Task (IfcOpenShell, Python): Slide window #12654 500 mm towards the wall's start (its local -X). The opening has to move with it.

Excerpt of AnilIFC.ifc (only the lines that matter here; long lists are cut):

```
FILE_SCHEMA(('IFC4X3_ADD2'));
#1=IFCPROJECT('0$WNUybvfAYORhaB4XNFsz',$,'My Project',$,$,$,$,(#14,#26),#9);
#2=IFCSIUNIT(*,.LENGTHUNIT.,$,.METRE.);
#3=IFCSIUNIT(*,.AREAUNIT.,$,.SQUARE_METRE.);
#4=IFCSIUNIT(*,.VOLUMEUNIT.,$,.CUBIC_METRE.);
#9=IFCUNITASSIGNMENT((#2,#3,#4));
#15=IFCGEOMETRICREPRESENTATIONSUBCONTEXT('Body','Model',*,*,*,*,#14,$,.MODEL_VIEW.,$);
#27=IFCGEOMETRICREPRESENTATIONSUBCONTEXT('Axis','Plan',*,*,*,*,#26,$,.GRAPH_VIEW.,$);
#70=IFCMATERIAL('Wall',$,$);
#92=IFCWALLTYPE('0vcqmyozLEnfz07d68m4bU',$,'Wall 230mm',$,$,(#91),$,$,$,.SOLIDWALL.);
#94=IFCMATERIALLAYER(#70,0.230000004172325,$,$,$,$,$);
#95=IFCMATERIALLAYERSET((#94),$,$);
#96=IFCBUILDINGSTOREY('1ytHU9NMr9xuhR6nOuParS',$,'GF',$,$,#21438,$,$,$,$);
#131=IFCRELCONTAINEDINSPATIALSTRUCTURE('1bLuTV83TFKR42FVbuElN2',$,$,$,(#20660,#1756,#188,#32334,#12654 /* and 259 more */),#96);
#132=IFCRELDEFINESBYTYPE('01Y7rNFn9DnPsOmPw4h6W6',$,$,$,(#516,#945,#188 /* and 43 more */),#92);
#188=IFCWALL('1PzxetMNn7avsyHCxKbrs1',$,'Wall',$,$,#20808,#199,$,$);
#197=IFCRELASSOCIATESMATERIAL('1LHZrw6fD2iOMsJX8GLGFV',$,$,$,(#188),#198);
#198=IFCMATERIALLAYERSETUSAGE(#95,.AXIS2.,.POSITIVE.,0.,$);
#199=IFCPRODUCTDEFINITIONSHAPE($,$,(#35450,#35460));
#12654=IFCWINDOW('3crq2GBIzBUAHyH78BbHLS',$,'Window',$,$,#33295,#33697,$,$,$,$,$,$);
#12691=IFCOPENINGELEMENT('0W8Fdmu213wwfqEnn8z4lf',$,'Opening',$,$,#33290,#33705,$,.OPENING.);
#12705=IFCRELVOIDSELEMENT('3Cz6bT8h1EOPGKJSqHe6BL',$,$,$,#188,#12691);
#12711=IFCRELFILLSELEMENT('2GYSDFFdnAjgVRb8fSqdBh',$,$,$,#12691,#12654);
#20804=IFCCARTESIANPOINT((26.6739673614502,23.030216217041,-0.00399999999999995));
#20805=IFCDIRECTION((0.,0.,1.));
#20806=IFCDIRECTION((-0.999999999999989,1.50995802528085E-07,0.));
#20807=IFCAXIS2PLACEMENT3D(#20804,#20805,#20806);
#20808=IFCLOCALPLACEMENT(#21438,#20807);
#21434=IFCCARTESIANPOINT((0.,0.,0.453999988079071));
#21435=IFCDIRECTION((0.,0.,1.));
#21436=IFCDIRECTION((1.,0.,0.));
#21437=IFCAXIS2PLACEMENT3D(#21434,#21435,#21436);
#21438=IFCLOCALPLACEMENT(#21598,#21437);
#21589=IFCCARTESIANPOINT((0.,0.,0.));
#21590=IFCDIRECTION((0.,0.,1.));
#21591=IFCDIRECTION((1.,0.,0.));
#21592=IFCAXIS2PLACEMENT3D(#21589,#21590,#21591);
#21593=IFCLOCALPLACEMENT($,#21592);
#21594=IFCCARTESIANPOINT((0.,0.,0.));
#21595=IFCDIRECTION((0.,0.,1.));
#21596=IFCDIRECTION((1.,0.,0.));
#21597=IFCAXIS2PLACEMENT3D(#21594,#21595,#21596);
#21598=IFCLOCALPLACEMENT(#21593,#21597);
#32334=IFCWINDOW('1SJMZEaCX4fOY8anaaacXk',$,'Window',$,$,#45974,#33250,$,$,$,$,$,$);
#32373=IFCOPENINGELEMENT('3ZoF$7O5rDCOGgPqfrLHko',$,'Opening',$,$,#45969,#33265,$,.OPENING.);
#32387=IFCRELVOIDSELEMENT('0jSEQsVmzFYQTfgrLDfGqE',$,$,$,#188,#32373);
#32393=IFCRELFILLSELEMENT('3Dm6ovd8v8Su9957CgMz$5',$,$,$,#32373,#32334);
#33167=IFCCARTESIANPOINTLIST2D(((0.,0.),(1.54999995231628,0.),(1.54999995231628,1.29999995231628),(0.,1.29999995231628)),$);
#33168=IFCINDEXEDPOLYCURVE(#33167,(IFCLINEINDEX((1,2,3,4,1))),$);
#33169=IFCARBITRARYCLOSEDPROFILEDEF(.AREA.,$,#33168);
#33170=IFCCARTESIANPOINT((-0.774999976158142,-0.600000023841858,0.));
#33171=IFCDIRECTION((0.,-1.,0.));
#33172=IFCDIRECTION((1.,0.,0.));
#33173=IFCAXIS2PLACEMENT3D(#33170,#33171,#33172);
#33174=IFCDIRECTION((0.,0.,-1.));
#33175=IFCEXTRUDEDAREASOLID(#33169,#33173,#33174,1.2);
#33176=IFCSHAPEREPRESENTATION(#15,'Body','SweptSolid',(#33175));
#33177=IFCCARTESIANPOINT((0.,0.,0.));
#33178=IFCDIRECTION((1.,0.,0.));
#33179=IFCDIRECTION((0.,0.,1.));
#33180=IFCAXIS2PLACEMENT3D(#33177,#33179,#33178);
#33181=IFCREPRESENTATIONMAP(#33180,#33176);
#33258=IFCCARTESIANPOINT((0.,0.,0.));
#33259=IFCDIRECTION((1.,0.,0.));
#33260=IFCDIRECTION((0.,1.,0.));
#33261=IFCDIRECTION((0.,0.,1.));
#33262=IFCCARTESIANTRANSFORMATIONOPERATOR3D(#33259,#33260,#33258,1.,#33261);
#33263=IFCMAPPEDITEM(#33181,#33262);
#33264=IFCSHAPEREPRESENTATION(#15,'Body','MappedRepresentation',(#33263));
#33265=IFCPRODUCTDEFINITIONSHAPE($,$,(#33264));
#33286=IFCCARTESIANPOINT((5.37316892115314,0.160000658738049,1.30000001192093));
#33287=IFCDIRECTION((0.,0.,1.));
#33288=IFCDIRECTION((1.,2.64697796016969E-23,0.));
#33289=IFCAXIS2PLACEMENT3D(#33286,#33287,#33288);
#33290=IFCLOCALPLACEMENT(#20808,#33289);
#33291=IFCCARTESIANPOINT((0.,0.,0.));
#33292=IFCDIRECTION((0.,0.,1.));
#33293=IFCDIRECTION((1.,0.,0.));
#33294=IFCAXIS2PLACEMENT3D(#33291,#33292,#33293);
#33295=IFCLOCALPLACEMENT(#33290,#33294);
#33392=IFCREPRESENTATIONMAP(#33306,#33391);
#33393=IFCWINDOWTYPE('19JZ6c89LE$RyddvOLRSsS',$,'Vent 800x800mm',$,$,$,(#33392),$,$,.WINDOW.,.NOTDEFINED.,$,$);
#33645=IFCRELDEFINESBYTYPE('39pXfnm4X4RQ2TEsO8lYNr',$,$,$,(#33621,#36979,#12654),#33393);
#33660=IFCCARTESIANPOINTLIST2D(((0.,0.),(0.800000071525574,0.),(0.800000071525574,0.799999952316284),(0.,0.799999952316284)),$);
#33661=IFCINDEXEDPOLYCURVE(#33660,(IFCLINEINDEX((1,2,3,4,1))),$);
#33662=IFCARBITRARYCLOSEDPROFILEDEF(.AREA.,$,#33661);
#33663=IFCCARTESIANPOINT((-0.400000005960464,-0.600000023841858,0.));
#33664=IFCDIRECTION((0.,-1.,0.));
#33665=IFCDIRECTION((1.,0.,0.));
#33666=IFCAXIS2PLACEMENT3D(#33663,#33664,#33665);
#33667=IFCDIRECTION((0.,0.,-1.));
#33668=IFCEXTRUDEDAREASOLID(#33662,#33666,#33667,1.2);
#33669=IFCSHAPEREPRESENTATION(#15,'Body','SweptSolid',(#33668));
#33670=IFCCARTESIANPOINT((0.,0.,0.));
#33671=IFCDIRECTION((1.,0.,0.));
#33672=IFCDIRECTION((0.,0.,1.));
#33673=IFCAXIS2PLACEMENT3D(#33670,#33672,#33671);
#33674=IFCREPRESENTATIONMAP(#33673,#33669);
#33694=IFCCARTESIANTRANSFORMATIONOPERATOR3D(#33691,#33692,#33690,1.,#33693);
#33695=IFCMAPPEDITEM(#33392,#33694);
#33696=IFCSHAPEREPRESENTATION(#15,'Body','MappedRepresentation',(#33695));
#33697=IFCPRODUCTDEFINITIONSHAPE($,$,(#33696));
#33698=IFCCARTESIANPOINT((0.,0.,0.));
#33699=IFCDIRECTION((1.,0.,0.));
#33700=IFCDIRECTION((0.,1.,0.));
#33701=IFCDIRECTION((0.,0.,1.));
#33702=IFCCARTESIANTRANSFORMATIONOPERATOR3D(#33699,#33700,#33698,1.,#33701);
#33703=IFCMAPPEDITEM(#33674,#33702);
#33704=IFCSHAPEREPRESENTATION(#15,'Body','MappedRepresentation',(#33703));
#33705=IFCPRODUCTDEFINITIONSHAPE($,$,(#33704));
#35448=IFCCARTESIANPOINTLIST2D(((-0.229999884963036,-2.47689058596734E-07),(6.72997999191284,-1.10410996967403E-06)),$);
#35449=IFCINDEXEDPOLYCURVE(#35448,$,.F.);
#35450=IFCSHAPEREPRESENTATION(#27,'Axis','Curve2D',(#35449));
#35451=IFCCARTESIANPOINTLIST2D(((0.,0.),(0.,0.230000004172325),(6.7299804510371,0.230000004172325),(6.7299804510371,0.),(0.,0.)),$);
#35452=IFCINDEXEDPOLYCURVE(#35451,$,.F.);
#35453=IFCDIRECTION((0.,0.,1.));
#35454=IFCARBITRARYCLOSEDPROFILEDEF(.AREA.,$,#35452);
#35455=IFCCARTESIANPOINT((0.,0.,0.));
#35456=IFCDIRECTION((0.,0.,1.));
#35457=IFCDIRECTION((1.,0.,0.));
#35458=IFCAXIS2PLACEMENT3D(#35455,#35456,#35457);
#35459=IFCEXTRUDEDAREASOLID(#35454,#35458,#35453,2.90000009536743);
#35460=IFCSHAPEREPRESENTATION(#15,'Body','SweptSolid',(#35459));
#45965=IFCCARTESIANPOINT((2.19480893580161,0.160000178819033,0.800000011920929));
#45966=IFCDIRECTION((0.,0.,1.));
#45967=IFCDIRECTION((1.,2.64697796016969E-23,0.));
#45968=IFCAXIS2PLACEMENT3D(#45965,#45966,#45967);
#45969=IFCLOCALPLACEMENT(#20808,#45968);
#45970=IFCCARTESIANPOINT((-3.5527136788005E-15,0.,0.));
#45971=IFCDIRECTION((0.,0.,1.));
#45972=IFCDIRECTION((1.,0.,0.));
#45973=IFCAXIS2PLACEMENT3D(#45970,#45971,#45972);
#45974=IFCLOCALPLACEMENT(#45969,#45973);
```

```python
import ifcopenshell
import ifcopenshell.api.geometry
import ifcopenshell.util.placement
import ifcopenshell.util.unit

model = ifcopenshell.open("AnilIFC.ifc")
unit_scale = ifcopenshell.util.unit.calculate_unit_scale(model)

window = model.by_guid("3crq2GBIzBUAHyH78BbHLS")
opening = window.FillsVoids[0].RelatingOpeningElement
wall = opening.VoidsElements[0].RelatingBuildingElement

wall_matrix = ifcopenshell.util.placement.get_local_placement(wall.ObjectPlacement)
shift = wall_matrix[:3, 0] * -0.5 / unit_scale
before = ifcopenshell.util.placement.get_local_placement(window.ObjectPlacement)[:3, 3].copy()

# The window is placed relative to its opening, so it follows when the opening moves.
matrix = ifcopenshell.util.placement.get_local_placement(opening.ObjectPlacement)
matrix[:3, 3] += shift
ifcopenshell.api.geometry.edit_object_placement(
    model, product=opening, matrix=matrix, is_si=False, should_transform_children=True
)

after = ifcopenshell.util.placement.get_local_placement(window.ObjectPlacement)[:3, 3]
print("window moved by", (after - before).round(3) + 0.0)

model.write("AnilIFC_rev.ifc")
```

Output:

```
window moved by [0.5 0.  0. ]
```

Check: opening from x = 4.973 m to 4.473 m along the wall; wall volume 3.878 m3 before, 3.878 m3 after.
